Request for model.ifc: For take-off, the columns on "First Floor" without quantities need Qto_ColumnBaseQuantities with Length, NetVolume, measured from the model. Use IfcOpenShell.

First a look at what the model holds.

```python
import ifcopenshell
import ifcopenshell.util.element
import ifcopenshell.util.unit

model = ifcopenshell.open("model.ifc")
print(model.schema)
for unit_type in ("LENGTHUNIT", "AREAUNIT", "VOLUMEUNIT"):
    print(unit_type, ifcopenshell.util.unit.calculate_unit_scale(model, unit_type))
storey = next(s for s in model.by_type("IfcBuildingStorey") if s.Name == "First Floor")
columns = [e for e in ifcopenshell.util.element.get_decomposition(storey) if e.is_a("IfcColumn")]
for e in sorted(columns, key=lambda e: e.id()):
    print(e.id(), e.is_a(), e.Name, list(ifcopenshell.util.element.get_psets(e, qtos_only=True)), sep=" | ")
```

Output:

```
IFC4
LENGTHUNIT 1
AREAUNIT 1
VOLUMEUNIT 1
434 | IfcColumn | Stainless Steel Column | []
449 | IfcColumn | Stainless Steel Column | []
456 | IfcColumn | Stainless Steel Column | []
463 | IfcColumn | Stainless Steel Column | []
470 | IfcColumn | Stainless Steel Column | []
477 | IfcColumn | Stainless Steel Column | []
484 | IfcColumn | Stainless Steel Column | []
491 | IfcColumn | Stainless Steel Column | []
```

```python
import ifcopenshell
import ifcopenshell.api.pset
import ifcopenshell.geom
import ifcopenshell.util.element
import ifcopenshell.util.shape
import ifcopenshell.util.unit

model = ifcopenshell.open("model.ifc")
unit_scale = ifcopenshell.util.unit.calculate_unit_scale(model)
volume_scale = ifcopenshell.util.unit.calculate_unit_scale(model, "VOLUMEUNIT")
settings = ifcopenshell.geom.settings()

storey = next(s for s in model.by_type("IfcBuildingStorey") if s.Name == "First Floor")
columns = [e for e in ifcopenshell.util.element.get_decomposition(storey) if e.is_a("IfcColumn")]

for e in sorted(columns, key=lambda e: e.id()):
    if ifcopenshell.util.element.get_psets(e, qtos_only=True, should_inherit=False):
        continue
    # Geometry comes back in metres, in the element's own axes.
    shape = ifcopenshell.geom.create_shape(settings, e)
    values = {
        "Length": ifcopenshell.util.shape.get_z(shape.geometry) / unit_scale,
        "NetVolume": ifcopenshell.util.shape.get_volume(shape.geometry) / volume_scale,
    }
    qto = ifcopenshell.api.pset.add_qto(model, product=e, name="Qto_ColumnBaseQuantities")
    ifcopenshell.api.pset.edit_qto(model, qto=qto, properties=values)
    print(e.id(), {k: round(v, 3) for k, v in values.items()})

model.write("model_rev.ifc")
```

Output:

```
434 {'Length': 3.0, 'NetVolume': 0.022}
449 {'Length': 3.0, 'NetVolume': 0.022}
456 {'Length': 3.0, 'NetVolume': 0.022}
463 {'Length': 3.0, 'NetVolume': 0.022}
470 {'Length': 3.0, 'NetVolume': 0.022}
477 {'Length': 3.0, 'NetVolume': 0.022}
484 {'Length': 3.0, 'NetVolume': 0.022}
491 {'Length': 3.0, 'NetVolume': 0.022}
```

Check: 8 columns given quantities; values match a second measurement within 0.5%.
